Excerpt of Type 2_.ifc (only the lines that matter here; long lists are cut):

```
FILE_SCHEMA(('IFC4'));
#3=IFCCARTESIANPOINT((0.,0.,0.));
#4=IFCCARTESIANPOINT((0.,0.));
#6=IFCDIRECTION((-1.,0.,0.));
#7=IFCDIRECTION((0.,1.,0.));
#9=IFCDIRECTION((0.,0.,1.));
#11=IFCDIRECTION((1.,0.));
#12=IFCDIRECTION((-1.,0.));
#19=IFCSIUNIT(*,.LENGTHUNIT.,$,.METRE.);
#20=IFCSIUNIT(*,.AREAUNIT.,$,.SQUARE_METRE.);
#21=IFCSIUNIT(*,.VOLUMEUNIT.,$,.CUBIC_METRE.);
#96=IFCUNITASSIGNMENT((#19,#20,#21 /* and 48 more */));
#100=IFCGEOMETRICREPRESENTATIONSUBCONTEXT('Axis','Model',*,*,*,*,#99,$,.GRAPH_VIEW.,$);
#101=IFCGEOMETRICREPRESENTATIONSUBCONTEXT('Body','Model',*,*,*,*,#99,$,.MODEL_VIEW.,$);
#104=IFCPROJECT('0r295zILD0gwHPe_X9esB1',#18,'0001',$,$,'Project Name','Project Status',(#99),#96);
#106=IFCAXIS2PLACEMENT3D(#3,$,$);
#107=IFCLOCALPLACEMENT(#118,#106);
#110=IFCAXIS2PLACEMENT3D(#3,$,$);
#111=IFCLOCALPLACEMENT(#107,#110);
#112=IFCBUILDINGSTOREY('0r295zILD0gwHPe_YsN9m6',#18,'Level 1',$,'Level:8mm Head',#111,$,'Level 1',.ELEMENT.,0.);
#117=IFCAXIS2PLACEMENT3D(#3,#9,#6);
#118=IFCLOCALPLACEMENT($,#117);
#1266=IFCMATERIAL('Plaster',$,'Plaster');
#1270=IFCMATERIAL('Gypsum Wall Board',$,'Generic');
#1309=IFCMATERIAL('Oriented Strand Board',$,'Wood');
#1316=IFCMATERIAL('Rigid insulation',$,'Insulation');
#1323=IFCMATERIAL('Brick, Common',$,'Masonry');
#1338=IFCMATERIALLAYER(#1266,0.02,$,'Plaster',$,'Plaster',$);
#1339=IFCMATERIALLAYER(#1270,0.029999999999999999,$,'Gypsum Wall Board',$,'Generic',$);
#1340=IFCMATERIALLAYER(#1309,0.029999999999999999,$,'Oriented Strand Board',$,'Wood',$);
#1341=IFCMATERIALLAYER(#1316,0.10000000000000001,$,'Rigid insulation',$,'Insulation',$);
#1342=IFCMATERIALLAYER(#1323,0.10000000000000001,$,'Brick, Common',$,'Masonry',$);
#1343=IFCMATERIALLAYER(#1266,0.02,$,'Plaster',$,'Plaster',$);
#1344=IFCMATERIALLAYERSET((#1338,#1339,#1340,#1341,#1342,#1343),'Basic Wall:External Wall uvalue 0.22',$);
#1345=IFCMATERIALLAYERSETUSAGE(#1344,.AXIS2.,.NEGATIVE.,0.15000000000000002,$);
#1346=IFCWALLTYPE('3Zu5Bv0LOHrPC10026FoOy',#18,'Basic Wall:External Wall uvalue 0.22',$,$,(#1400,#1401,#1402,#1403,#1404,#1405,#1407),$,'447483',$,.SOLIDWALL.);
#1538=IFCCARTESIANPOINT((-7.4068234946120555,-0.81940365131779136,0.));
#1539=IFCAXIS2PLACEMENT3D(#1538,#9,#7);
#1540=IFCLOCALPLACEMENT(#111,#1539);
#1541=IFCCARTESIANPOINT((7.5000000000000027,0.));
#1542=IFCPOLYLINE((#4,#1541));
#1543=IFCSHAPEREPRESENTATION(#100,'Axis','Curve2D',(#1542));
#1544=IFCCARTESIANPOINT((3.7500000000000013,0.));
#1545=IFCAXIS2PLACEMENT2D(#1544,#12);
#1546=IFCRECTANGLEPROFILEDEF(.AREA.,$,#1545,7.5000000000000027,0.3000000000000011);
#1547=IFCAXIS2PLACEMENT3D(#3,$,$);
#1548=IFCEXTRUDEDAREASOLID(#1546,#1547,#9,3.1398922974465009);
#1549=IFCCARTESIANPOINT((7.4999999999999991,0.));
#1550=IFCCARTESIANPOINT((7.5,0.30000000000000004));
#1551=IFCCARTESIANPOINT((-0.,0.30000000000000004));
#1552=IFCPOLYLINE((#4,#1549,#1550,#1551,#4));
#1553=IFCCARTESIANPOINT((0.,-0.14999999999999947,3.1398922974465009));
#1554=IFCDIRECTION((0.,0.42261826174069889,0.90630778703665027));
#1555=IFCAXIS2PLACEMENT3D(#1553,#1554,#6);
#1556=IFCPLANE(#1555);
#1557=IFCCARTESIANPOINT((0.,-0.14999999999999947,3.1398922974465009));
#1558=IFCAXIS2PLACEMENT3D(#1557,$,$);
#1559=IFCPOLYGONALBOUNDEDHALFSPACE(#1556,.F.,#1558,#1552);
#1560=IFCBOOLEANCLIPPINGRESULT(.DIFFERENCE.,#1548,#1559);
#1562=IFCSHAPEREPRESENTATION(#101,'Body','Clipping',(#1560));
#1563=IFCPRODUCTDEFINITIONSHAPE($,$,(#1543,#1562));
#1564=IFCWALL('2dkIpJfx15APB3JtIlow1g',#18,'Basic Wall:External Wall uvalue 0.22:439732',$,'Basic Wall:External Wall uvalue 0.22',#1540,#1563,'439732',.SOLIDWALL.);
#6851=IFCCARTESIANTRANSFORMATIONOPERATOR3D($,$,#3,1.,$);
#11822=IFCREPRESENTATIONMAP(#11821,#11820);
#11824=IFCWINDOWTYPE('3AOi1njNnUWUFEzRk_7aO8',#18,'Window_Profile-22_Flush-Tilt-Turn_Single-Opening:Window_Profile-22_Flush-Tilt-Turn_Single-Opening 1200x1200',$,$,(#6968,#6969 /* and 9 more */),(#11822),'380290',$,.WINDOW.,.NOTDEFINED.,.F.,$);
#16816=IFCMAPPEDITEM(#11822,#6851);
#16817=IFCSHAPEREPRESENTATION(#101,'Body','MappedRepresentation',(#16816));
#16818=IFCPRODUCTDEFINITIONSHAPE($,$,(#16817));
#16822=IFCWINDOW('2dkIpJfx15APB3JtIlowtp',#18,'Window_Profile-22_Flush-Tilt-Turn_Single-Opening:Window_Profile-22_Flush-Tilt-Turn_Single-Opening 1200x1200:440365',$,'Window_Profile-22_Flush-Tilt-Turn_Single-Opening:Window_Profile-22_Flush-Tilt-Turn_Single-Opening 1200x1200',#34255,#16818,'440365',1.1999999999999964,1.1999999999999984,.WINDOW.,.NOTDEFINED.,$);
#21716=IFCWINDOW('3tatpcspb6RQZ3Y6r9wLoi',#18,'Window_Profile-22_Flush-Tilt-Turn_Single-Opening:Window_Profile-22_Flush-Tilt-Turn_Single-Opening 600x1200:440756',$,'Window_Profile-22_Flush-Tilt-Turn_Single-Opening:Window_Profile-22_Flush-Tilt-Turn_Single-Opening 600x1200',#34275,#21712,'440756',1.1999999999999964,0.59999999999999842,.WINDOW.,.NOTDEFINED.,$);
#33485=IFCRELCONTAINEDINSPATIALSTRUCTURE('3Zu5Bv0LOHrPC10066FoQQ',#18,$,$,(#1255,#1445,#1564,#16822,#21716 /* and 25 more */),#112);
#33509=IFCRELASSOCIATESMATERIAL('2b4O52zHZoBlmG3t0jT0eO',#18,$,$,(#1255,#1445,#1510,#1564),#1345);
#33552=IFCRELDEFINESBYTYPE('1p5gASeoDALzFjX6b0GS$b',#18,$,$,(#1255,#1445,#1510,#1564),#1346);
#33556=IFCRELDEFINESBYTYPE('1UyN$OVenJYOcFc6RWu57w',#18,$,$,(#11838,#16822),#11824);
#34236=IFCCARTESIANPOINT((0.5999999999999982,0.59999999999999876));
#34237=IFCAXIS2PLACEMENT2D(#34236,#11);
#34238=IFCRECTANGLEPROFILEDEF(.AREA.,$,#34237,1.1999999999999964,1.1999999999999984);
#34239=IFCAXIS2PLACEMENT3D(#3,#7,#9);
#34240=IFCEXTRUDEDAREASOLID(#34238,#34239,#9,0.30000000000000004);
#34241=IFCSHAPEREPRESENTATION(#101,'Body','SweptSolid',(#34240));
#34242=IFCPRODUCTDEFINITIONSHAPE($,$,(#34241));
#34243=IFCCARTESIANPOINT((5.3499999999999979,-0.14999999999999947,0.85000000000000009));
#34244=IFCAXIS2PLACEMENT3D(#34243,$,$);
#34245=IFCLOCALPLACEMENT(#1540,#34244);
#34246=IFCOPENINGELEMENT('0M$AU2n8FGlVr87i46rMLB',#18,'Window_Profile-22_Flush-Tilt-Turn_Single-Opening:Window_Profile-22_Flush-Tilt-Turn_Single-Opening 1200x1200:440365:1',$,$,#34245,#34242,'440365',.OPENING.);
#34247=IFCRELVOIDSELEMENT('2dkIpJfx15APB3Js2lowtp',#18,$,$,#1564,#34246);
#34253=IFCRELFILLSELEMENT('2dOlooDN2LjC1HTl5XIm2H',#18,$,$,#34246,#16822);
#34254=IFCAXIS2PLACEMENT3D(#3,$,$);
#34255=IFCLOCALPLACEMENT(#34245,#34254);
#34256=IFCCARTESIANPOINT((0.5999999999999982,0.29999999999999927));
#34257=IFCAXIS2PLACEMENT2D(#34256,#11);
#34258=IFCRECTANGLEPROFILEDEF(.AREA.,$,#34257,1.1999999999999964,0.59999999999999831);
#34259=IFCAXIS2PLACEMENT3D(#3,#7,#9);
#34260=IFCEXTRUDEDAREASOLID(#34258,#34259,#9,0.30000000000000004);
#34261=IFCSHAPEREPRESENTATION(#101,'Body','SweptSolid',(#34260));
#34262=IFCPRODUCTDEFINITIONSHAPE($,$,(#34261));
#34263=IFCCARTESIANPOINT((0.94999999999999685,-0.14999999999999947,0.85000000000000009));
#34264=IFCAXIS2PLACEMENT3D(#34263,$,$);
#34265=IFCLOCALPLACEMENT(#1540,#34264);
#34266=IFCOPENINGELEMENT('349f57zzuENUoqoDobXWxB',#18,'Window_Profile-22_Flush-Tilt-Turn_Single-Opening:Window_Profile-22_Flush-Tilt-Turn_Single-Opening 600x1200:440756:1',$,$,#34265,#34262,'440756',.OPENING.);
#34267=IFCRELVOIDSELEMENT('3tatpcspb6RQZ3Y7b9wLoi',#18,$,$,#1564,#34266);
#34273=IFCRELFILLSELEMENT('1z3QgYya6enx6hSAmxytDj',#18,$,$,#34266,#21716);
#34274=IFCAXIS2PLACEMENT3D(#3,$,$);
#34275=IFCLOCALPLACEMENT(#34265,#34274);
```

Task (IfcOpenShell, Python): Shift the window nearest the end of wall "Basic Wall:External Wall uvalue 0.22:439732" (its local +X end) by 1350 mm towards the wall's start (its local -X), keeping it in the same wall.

```python
import ifcopenshell
import ifcopenshell.api.geometry
import ifcopenshell.util.placement

model = ifcopenshell.open("Type 2_.ifc")

window = model.by_guid("2dkIpJfx15APB3JtIlowtp")
opening = window.FillsVoids[0].RelatingOpeningElement
wall = opening.VoidsElements[0].RelatingBuildingElement

wall_matrix = ifcopenshell.util.placement.get_local_placement(wall.ObjectPlacement)
shift = wall_matrix[:3, 0] * -1.35
before = ifcopenshell.util.placement.get_local_placement(window.ObjectPlacement)[:3, 3].copy()

# The window is placed relative to its opening, so it follows when the opening moves.
matrix = ifcopenshell.util.placement.get_local_placement(opening.ObjectPlacement)
matrix[:3, 3] += shift
ifcopenshell.api.geometry.edit_object_placement(
    model, product=opening, matrix=matrix, is_si=False, should_transform_children=True
)

after = ifcopenshell.util.placement.get_local_placement(window.ObjectPlacement)[:3, 3]
print("window moved by", (after - before).round(3) + 0.0)

model.write("Type 2__updated.ifc")
```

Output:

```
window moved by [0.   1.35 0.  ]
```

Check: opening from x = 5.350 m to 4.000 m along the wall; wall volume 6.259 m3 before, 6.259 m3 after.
